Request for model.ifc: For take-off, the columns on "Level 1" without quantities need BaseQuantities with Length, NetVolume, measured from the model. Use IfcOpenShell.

First a look at what the model holds.

```python
import ifcopenshell
import ifcopenshell.util.element
import ifcopenshell.util.unit

model = ifcopenshell.open("model.ifc")
print(model.schema)
for unit_type in ("LENGTHUNIT", "AREAUNIT", "VOLUMEUNIT"):
    print(unit_type, ifcopenshell.util.unit.calculate_unit_scale(model, unit_type))
storey = next(s for s in model.by_type("IfcBuildingStorey") if s.Name == "Level 1")
columns = [e for e in ifcopenshell.util.element.get_decomposition(storey) if e.is_a("IfcColumn")]
for e in sorted(columns, key=lambda e: e.id()):
    print(e.id(), e.is_a(), e.Name, list(ifcopenshell.util.element.get_psets(e, qtos_only=True)), sep=" | ")
```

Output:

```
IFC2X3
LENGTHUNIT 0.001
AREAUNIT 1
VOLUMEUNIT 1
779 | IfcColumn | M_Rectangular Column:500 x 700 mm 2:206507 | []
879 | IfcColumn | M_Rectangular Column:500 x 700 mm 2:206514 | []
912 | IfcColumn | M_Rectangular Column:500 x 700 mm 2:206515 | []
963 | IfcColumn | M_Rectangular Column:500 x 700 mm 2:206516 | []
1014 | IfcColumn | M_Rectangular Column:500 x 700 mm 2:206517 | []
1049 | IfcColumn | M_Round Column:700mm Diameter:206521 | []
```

```python
import ifcopenshell
import ifcopenshell.api.pset
import ifcopenshell.geom
import ifcopenshell.util.element
import ifcopenshell.util.shape
import ifcopenshell.util.unit

model = ifcopenshell.open("model.ifc")
unit_scale = ifcopenshell.util.unit.calculate_unit_scale(model)
volume_scale = ifcopenshell.util.unit.calculate_unit_scale(model, "VOLUMEUNIT")
settings = ifcopenshell.geom.settings()

storey = next(s for s in model.by_type("IfcBuildingStorey") if s.Name == "Level 1")
columns = [e for e in ifcopenshell.util.element.get_decomposition(storey) if e.is_a("IfcColumn")]

for e in sorted(columns, key=lambda e: e.id()):
    if ifcopenshell.util.element.get_psets(e, qtos_only=True, should_inherit=False):
        continue
    # Geometry comes back in metres, in the element's own axes.
    shape = ifcopenshell.geom.create_shape(settings, e)
    values = {
        "Length": ifcopenshell.util.shape.get_z(shape.geometry) / unit_scale,
        "NetVolume": ifcopenshell.util.shape.get_volume(shape.geometry) / volume_scale,
    }
    qto = ifcopenshell.api.pset.add_qto(model, product=e, name="BaseQuantities")
    ifcopenshell.api.pset.edit_qto(model, qto=qto, properties=values)
    print(e.id(), {k: round(v, 3) for k, v in values.items()})

model.write("model_v2.ifc")
```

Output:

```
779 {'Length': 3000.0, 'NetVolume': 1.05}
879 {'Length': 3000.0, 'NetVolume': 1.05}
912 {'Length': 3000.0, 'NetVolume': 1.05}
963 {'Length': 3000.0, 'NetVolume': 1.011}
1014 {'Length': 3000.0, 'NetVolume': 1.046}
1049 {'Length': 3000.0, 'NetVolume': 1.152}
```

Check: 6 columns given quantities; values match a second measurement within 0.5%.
